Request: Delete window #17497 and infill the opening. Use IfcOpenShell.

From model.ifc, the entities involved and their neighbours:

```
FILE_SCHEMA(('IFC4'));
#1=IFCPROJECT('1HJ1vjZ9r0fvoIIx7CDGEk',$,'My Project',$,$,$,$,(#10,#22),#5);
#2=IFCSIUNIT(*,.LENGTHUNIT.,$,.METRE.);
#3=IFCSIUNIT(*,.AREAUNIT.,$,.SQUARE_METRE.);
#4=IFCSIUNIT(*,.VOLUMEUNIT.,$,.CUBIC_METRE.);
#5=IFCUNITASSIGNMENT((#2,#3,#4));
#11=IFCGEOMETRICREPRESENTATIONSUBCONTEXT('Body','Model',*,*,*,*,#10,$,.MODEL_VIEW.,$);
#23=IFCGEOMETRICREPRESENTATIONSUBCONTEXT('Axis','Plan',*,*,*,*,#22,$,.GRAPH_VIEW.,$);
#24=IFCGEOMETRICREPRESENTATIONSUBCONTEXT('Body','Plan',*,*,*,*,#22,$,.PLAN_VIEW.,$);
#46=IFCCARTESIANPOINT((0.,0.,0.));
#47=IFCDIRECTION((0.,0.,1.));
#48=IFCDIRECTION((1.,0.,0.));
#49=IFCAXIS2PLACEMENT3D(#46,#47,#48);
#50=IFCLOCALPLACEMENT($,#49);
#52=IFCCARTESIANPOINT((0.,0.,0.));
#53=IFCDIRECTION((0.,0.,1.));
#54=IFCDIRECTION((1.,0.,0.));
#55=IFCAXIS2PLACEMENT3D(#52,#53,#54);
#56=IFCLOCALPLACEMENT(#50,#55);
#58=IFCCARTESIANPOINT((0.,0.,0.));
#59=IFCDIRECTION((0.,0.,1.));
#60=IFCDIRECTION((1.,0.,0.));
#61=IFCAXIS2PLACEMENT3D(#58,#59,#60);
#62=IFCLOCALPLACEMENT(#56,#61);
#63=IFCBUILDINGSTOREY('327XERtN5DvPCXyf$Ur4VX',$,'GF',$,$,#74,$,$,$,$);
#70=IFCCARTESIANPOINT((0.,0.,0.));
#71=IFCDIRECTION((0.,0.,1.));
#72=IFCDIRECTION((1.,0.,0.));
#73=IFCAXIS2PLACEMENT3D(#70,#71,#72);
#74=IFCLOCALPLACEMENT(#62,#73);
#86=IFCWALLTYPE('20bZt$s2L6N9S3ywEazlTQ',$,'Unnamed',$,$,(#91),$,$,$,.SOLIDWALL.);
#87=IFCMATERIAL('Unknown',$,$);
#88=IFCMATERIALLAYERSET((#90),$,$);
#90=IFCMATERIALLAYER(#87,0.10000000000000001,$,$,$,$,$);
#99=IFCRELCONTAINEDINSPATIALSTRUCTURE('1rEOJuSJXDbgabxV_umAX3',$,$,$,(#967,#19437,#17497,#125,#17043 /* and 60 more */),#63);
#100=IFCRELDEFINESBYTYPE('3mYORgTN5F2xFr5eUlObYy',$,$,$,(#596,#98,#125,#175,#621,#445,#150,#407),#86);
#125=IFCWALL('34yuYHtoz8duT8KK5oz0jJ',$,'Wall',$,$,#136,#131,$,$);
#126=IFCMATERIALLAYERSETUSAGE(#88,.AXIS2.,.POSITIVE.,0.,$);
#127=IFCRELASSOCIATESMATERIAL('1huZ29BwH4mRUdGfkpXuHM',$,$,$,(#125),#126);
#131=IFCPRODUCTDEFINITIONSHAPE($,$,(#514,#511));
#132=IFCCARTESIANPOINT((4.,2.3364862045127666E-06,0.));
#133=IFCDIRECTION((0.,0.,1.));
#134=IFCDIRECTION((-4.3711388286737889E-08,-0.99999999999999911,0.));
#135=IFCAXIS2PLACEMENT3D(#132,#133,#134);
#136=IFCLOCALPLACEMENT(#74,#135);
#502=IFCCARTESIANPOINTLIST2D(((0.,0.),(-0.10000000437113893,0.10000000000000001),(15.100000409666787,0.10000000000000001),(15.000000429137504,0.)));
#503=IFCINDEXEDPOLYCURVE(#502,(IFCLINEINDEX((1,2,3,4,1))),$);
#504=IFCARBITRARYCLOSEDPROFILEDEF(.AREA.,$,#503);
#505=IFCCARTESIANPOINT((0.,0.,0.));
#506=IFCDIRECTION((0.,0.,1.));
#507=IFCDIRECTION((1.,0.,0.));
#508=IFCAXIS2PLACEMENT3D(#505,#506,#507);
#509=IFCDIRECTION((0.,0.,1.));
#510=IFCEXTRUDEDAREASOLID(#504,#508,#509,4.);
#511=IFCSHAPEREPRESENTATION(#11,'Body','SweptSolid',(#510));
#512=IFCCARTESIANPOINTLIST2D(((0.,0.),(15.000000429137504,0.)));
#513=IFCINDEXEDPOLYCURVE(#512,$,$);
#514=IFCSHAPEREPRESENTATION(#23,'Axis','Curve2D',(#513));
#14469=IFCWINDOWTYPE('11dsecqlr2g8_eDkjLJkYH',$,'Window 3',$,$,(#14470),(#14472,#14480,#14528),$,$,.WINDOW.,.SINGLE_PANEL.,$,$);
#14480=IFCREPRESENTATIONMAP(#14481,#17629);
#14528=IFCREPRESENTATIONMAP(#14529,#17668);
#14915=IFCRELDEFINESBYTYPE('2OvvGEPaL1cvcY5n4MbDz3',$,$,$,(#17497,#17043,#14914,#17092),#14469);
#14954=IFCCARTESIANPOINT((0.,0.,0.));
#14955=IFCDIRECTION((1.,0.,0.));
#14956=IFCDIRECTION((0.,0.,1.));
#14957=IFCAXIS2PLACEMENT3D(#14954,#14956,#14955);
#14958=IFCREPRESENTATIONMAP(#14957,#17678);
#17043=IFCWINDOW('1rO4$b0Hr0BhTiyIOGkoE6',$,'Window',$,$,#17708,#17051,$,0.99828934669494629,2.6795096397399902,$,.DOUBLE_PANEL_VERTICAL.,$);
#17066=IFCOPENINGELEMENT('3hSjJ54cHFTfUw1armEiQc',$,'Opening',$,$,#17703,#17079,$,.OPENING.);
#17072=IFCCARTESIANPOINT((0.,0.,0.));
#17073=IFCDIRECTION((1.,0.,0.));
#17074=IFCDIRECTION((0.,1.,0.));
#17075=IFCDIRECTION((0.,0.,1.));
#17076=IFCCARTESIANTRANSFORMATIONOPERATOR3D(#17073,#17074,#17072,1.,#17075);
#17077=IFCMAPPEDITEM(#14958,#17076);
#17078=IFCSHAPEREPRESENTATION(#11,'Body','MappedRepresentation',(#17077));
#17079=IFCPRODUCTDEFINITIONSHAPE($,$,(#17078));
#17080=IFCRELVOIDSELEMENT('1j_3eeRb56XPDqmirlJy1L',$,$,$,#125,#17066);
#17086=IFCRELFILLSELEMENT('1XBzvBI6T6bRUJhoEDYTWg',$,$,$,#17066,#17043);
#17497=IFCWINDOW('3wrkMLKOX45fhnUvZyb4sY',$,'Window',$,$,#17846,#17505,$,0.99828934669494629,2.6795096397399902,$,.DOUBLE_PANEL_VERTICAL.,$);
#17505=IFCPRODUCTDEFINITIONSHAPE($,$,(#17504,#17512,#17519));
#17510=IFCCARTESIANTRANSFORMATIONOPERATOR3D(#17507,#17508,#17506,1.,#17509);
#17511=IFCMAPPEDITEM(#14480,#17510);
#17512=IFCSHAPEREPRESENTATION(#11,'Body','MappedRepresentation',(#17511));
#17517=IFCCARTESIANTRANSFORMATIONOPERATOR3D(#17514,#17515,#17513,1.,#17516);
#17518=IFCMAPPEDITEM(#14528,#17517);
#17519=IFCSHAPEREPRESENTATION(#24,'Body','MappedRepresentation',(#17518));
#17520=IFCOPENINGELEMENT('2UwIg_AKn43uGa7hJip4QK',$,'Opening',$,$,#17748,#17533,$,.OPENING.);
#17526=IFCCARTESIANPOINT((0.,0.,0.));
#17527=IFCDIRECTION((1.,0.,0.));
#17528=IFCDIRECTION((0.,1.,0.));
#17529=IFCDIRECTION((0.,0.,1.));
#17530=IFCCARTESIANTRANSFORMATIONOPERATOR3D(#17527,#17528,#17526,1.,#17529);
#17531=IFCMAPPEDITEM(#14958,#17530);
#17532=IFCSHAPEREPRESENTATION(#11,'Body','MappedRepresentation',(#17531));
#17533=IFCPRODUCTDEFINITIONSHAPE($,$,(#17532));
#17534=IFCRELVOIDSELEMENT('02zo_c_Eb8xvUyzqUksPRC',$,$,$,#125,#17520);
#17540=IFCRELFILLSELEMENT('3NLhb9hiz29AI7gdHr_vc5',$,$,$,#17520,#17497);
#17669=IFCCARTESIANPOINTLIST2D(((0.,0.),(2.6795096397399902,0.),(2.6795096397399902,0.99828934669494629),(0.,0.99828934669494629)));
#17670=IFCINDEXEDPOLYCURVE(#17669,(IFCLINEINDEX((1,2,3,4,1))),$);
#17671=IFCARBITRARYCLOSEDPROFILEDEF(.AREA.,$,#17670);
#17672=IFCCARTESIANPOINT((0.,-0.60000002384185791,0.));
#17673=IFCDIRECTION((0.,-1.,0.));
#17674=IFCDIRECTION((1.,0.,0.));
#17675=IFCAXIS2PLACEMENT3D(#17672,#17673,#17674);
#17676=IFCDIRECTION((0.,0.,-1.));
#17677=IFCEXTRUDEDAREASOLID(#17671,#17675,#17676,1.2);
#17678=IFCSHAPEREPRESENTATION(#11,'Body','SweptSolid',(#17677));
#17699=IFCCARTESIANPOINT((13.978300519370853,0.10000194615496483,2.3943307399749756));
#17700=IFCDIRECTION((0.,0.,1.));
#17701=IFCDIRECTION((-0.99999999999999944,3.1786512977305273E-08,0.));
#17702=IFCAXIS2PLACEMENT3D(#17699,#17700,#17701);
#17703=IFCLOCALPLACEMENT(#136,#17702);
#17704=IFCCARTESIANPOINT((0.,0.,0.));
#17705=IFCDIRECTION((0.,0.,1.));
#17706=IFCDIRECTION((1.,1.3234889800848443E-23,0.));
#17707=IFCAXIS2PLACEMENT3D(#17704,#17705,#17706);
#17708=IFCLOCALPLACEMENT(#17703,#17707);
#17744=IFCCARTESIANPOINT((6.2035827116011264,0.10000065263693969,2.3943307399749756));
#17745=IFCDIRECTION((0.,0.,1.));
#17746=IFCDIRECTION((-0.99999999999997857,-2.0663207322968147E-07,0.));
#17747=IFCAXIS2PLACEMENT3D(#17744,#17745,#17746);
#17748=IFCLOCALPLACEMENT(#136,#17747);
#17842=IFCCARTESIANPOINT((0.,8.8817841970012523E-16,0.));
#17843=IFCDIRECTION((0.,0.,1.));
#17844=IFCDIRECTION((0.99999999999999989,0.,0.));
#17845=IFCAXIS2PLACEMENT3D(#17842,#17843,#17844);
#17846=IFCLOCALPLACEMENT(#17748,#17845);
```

```python
import ifcopenshell
import ifcopenshell.api.feature
import ifcopenshell.api.root
import ifcopenshell.geom
import ifcopenshell.util.shape

model = ifcopenshell.open("model.ifc")
settings = ifcopenshell.geom.settings()


def volume(element):
    """Net volume in cubic metres, openings subtracted."""
    shape = ifcopenshell.geom.create_shape(settings, element)
    return ifcopenshell.util.shape.get_volume(shape.geometry)


window = model.by_guid("3wrkMLKOX45fhnUvZyb4sY")
opening = window.FillsVoids[0].RelatingOpeningElement
wall = opening.VoidsElements[0].RelatingBuildingElement
before = volume(wall)

ifcopenshell.api.root.remove_product(model, product=window)
ifcopenshell.api.feature.remove_feature(model, feature=opening)

after = volume(wall)

print(f"wall volume {before:.3f} -> {after:.3f} m3")

model.write("model_updated.ifc")
```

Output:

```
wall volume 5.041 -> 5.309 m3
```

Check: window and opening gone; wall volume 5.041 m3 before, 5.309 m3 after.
